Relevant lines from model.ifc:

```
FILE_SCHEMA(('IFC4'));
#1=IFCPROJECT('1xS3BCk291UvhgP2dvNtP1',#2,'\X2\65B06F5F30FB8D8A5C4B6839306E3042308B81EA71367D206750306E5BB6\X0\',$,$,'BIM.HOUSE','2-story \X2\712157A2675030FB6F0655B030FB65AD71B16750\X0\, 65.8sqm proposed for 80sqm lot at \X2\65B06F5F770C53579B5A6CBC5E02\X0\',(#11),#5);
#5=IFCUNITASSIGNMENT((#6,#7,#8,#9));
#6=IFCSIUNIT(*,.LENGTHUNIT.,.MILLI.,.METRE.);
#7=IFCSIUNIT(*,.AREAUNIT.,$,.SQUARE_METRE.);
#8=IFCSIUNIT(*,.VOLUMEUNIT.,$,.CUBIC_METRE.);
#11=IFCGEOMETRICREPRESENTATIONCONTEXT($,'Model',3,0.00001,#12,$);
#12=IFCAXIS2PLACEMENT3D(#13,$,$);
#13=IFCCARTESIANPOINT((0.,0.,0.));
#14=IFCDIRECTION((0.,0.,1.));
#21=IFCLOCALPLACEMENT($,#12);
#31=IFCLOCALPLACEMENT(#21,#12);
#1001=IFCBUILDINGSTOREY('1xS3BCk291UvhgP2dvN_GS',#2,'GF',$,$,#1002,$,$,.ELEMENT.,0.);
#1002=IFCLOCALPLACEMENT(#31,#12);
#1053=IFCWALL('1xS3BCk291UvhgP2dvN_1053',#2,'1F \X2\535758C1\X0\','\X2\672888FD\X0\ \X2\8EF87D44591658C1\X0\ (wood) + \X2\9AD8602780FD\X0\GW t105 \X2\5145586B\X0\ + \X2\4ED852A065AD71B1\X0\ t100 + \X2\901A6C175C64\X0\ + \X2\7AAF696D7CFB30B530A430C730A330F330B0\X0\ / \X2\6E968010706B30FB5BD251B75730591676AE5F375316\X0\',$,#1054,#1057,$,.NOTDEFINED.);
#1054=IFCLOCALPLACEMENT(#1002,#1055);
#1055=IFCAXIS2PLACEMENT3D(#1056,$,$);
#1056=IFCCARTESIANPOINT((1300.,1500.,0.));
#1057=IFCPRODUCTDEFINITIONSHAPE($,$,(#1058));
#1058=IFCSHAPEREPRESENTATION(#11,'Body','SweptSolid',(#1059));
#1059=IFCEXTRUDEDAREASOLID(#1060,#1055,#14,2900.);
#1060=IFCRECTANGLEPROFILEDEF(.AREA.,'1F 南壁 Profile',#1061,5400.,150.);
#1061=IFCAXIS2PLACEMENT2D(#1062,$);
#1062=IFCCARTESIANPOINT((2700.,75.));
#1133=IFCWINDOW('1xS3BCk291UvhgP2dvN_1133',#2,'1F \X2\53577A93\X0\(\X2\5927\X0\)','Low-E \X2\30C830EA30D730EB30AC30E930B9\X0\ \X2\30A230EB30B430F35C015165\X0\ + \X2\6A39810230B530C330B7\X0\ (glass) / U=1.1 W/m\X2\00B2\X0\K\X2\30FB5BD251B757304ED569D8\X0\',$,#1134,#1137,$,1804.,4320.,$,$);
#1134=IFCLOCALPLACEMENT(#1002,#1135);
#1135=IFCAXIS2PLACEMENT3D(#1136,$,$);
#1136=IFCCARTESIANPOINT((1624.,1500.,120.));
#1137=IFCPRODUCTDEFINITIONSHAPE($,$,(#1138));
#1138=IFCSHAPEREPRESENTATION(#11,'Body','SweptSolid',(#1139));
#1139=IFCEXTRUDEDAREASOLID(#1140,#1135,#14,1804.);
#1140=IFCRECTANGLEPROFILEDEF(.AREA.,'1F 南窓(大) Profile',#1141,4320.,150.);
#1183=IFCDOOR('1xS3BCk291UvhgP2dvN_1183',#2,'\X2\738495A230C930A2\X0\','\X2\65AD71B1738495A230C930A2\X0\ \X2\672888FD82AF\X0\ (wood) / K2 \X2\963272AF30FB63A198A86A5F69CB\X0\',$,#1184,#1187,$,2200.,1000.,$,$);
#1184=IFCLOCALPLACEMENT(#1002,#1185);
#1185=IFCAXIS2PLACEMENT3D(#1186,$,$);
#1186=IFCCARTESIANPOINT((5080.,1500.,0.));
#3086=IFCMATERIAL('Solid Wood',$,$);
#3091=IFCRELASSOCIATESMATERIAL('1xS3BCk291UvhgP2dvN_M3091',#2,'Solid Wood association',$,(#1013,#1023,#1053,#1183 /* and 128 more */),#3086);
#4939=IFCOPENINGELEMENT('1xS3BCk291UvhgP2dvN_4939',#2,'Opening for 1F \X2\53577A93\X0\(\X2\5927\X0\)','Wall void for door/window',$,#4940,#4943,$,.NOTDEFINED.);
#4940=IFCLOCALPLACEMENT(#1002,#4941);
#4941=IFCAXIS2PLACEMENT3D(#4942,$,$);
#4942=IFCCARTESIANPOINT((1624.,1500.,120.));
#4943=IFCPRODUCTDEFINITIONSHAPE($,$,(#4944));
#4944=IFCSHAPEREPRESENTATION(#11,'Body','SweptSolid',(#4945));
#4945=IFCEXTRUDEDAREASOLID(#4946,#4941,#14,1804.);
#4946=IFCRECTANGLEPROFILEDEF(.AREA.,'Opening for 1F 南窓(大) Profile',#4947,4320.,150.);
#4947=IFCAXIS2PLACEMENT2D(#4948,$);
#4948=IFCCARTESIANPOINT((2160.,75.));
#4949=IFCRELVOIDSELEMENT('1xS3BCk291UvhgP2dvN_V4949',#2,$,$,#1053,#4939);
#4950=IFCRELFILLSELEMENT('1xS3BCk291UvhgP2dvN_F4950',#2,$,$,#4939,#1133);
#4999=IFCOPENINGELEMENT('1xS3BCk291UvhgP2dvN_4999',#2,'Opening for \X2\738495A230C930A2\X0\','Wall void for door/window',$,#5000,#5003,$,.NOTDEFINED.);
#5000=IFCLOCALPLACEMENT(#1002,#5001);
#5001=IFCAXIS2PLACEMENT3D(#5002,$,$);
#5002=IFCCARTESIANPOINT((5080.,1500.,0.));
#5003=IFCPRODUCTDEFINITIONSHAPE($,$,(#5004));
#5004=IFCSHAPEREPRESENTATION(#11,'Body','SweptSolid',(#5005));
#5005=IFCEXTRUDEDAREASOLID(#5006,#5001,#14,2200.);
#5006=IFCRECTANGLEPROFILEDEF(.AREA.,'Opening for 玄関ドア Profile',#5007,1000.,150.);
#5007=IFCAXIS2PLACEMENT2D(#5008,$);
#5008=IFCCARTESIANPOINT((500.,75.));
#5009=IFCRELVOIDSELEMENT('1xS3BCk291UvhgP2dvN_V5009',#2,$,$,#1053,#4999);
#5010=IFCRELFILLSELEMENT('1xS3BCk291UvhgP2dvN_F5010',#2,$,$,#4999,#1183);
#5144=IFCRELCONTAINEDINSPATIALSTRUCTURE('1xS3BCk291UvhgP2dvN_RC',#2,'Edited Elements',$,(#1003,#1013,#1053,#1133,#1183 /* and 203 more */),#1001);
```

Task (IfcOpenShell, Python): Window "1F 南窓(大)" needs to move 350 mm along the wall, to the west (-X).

```python
import ifcopenshell
import ifcopenshell.api.geometry
import ifcopenshell.util.placement
import ifcopenshell.util.unit

model = ifcopenshell.open("model.ifc")
unit_scale = ifcopenshell.util.unit.calculate_unit_scale(model)

window = model.by_id(1133)
opening = window.FillsVoids[0].RelatingOpeningElement
wall = opening.VoidsElements[0].RelatingBuildingElement

wall_matrix = ifcopenshell.util.placement.get_local_placement(wall.ObjectPlacement)
shift = wall_matrix[:3, 0] * -0.35 / unit_scale
before = ifcopenshell.util.placement.get_local_placement(window.ObjectPlacement)[:3, 3].copy()

# The window is not placed relative to its opening, so move both.
for product in (opening, window):
    matrix = ifcopenshell.util.placement.get_local_placement(product.ObjectPlacement)
    matrix[:3, 3] += shift
    ifcopenshell.api.geometry.edit_object_placement(model, product=product, matrix=matrix, is_si=False)

after = ifcopenshell.util.placement.get_local_placement(window.ObjectPlacement)[:3, 3]
print("window moved by", (after - before).round(3) + 0.0)

model.write("model_edited.ifc")
```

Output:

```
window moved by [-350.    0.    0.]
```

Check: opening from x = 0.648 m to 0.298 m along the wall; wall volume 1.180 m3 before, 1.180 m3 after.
